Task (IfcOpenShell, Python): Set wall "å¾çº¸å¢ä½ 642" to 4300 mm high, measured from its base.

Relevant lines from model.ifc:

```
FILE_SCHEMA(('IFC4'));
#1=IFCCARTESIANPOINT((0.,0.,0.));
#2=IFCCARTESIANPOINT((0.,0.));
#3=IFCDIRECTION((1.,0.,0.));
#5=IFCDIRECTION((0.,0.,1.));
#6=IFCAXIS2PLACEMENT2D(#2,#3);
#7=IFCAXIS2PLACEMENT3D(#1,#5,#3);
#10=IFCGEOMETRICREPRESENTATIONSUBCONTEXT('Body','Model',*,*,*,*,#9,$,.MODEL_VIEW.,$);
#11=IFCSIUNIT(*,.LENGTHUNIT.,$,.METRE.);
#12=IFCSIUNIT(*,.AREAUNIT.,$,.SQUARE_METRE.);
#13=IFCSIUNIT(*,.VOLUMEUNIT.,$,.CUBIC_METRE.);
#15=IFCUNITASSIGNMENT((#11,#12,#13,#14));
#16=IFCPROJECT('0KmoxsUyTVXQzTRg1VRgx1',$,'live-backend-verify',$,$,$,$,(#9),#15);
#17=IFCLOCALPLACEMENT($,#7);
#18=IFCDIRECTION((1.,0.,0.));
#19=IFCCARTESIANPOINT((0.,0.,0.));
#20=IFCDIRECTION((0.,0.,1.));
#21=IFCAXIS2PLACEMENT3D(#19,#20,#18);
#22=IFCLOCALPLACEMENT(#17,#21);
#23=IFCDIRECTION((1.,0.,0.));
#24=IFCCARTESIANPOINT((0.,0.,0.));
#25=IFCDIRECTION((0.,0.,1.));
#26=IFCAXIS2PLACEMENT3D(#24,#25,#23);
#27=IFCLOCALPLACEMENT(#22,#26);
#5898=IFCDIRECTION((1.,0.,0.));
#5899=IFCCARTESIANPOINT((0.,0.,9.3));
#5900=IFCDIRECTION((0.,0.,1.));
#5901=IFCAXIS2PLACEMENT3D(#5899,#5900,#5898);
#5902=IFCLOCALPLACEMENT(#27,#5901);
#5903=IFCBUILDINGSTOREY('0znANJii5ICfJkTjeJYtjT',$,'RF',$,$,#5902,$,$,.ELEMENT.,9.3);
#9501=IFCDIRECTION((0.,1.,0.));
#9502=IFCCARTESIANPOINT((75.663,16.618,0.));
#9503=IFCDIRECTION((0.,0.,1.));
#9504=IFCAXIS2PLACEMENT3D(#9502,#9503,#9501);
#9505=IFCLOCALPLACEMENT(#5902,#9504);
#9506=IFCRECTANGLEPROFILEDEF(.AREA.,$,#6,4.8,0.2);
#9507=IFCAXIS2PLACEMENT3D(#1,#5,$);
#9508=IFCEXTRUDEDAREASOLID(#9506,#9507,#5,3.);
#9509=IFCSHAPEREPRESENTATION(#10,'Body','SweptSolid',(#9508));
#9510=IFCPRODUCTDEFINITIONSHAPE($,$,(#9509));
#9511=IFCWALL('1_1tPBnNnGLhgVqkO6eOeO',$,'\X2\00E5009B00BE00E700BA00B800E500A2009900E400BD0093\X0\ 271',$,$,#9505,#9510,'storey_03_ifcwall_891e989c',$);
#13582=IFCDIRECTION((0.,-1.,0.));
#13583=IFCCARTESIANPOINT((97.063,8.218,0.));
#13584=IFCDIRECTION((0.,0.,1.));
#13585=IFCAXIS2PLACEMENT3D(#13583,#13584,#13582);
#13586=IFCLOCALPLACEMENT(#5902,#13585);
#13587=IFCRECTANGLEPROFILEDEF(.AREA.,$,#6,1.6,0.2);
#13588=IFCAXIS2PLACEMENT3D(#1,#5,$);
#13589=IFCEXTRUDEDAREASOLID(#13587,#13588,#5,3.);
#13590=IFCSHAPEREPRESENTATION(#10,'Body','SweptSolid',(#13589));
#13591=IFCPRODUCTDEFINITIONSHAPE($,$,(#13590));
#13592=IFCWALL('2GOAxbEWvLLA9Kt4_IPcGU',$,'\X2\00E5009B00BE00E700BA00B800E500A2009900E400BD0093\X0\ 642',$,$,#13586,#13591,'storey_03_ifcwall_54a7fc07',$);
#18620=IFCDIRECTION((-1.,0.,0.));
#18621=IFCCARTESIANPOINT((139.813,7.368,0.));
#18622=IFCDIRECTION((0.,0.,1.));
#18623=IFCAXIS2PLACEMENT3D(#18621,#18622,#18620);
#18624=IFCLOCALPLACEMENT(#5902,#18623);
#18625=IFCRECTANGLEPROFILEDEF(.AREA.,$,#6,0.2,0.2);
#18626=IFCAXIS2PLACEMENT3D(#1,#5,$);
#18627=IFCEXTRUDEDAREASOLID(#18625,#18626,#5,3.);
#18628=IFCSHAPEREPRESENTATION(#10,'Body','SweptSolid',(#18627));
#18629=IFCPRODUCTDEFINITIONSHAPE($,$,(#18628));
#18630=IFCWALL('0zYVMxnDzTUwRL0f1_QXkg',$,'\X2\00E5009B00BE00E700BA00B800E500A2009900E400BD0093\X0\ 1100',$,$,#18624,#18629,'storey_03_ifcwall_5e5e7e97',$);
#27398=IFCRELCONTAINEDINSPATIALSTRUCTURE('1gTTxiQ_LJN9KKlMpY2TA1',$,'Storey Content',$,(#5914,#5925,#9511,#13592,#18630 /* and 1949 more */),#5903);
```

```python
import ifcopenshell
import ifcopenshell.geom
import ifcopenshell.util.representation
import ifcopenshell.util.shape

model = ifcopenshell.open("model.ifc")
settings = ifcopenshell.geom.settings()


def volume(element):
    """Net volume in cubic metres, openings subtracted."""
    shape = ifcopenshell.geom.create_shape(settings, element)
    return ifcopenshell.util.shape.get_volume(shape.geometry)


wall = model.by_id(13592)
before = volume(wall)

body = ifcopenshell.util.representation.get_representation(wall, "Model", "Body")
solid = body.Items[0]
old_height = solid.Depth
solid.Depth = 4.3
after = volume(wall)

print(f"height {old_height:g} -> {solid.Depth:g}, volume {before:.3f} -> {after:.3f} m3")

model.write("model_rev.ifc")
```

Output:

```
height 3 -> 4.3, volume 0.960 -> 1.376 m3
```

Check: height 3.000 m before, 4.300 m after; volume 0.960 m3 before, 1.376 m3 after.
